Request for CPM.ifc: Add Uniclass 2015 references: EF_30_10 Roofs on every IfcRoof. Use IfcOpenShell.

First a look at what the model holds.

```python
import ifcopenshell

model = ifcopenshell.open("CPM.ifc")
print(model.schema)
print("classifications:", [c.Name for c in model.by_type("IfcClassification")])
for ifc_class in ("IfcDoor", "IfcRoof", "IfcStair", "IfcWall", "IfcWindow"):
    print(ifc_class, len(model.by_type(ifc_class)))
```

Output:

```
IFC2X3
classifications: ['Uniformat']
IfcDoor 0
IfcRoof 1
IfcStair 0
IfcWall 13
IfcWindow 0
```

```python
import ifcopenshell
import ifcopenshell.api.classification

model = ifcopenshell.open("CPM.ifc")

# IFC2X3 requires Source and Edition and has no link from the project to the system.
system = model.create_entity("IfcClassification", Source="NBS", Edition="2015", Name="Uniclass 2015")

codes = {
    "IfcRoof": ("EF_30_10", "Roofs"),
}
for ifc_class, (code, name) in codes.items():
    products = model.by_type(ifc_class)
    ifcopenshell.api.classification.add_reference(
        model, products=products, classification=system, identification=code, name=name
    )
    print(code, len(products))

model.write("CPM_updated.ifc")
```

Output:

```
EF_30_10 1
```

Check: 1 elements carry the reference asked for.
